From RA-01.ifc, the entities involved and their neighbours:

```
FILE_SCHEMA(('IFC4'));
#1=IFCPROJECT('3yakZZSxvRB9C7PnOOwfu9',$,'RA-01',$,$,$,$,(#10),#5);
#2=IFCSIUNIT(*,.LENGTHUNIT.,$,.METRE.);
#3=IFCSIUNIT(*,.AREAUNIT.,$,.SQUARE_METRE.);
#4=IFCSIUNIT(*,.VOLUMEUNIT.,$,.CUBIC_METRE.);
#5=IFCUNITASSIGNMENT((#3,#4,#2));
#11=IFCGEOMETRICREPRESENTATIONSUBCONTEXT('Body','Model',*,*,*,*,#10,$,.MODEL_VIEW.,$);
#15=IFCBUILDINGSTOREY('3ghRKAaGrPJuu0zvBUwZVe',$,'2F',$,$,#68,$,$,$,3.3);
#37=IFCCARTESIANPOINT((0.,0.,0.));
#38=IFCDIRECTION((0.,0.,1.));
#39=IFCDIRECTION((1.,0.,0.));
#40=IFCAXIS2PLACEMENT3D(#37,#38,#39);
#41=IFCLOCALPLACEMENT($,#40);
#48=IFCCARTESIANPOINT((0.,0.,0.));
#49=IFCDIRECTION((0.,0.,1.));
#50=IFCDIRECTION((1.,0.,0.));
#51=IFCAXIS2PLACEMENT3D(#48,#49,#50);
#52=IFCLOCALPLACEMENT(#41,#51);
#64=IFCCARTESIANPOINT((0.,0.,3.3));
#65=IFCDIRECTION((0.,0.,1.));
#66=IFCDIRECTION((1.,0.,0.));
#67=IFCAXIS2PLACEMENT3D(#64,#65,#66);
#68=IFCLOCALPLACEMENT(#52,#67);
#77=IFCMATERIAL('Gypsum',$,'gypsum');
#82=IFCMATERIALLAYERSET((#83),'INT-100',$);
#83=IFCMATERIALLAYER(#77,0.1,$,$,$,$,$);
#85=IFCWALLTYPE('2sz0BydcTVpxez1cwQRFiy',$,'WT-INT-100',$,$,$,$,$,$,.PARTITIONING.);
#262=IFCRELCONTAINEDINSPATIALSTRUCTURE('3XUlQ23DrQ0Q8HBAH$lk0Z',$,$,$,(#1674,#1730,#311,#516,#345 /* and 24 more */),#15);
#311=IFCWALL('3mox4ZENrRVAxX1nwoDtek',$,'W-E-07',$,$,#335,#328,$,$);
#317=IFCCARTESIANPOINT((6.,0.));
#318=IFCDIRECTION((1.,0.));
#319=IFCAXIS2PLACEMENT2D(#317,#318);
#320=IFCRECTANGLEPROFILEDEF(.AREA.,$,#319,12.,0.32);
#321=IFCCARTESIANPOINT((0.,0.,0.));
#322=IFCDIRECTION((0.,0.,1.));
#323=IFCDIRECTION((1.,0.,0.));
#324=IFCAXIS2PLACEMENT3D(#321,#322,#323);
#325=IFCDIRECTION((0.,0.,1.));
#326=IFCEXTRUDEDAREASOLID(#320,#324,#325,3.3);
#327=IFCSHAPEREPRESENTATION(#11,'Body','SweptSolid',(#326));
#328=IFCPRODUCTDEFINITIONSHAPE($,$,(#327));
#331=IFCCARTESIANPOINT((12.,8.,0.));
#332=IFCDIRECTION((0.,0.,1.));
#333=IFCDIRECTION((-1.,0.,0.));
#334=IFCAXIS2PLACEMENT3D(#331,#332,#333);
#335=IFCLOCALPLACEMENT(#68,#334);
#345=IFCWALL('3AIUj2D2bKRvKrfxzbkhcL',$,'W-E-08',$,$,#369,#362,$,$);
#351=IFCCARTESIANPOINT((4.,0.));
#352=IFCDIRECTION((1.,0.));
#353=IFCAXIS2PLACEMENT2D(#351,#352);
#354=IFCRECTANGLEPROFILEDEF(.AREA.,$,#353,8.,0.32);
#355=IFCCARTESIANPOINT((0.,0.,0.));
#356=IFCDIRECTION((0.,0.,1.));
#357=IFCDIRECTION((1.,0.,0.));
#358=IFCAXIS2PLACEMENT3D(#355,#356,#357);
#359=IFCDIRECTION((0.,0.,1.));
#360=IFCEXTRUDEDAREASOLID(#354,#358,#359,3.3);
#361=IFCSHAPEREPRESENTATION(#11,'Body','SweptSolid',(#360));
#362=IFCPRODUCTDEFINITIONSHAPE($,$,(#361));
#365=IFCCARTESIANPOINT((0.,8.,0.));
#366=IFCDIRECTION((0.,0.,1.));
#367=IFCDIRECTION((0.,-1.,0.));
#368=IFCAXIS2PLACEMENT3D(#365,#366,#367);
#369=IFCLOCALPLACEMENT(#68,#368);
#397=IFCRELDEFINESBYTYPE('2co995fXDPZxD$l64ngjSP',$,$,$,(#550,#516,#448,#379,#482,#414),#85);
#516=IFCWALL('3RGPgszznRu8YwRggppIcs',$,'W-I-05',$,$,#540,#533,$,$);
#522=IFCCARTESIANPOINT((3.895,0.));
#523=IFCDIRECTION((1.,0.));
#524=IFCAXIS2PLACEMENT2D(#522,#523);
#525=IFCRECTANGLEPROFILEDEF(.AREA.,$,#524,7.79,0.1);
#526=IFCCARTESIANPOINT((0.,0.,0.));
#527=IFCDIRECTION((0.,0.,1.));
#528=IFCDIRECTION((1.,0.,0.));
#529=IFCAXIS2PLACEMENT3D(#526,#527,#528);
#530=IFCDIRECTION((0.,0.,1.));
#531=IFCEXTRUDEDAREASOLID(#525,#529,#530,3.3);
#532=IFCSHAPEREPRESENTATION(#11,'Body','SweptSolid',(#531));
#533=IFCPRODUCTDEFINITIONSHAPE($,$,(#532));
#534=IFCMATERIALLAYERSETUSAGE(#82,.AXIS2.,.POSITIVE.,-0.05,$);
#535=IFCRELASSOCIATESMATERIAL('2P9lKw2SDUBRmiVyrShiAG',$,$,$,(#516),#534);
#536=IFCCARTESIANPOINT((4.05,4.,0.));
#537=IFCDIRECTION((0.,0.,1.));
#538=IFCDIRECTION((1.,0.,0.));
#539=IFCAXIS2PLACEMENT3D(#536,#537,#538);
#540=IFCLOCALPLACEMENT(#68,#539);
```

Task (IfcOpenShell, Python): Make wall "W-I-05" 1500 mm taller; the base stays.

```python
import ifcopenshell
import ifcopenshell.geom
import ifcopenshell.util.representation
import ifcopenshell.util.shape

model = ifcopenshell.open("RA-01.ifc")
settings = ifcopenshell.geom.settings()


def volume(element):
    """Net volume in cubic metres, openings subtracted."""
    shape = ifcopenshell.geom.create_shape(settings, element)
    return ifcopenshell.util.shape.get_volume(shape.geometry)


wall = model.by_id(516)
before = volume(wall)

body = ifcopenshell.util.representation.get_representation(wall, "Model", "Body")
solid = body.Items[0]
old_height = solid.Depth
solid.Depth += 1.5
after = volume(wall)

print(f"height {old_height:g} -> {solid.Depth:g}, volume {before:.3f} -> {after:.3f} m3")

model.write("RA-01_v2.ifc")
```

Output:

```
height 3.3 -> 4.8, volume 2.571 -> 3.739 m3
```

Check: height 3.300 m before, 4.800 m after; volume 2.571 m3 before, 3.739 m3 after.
